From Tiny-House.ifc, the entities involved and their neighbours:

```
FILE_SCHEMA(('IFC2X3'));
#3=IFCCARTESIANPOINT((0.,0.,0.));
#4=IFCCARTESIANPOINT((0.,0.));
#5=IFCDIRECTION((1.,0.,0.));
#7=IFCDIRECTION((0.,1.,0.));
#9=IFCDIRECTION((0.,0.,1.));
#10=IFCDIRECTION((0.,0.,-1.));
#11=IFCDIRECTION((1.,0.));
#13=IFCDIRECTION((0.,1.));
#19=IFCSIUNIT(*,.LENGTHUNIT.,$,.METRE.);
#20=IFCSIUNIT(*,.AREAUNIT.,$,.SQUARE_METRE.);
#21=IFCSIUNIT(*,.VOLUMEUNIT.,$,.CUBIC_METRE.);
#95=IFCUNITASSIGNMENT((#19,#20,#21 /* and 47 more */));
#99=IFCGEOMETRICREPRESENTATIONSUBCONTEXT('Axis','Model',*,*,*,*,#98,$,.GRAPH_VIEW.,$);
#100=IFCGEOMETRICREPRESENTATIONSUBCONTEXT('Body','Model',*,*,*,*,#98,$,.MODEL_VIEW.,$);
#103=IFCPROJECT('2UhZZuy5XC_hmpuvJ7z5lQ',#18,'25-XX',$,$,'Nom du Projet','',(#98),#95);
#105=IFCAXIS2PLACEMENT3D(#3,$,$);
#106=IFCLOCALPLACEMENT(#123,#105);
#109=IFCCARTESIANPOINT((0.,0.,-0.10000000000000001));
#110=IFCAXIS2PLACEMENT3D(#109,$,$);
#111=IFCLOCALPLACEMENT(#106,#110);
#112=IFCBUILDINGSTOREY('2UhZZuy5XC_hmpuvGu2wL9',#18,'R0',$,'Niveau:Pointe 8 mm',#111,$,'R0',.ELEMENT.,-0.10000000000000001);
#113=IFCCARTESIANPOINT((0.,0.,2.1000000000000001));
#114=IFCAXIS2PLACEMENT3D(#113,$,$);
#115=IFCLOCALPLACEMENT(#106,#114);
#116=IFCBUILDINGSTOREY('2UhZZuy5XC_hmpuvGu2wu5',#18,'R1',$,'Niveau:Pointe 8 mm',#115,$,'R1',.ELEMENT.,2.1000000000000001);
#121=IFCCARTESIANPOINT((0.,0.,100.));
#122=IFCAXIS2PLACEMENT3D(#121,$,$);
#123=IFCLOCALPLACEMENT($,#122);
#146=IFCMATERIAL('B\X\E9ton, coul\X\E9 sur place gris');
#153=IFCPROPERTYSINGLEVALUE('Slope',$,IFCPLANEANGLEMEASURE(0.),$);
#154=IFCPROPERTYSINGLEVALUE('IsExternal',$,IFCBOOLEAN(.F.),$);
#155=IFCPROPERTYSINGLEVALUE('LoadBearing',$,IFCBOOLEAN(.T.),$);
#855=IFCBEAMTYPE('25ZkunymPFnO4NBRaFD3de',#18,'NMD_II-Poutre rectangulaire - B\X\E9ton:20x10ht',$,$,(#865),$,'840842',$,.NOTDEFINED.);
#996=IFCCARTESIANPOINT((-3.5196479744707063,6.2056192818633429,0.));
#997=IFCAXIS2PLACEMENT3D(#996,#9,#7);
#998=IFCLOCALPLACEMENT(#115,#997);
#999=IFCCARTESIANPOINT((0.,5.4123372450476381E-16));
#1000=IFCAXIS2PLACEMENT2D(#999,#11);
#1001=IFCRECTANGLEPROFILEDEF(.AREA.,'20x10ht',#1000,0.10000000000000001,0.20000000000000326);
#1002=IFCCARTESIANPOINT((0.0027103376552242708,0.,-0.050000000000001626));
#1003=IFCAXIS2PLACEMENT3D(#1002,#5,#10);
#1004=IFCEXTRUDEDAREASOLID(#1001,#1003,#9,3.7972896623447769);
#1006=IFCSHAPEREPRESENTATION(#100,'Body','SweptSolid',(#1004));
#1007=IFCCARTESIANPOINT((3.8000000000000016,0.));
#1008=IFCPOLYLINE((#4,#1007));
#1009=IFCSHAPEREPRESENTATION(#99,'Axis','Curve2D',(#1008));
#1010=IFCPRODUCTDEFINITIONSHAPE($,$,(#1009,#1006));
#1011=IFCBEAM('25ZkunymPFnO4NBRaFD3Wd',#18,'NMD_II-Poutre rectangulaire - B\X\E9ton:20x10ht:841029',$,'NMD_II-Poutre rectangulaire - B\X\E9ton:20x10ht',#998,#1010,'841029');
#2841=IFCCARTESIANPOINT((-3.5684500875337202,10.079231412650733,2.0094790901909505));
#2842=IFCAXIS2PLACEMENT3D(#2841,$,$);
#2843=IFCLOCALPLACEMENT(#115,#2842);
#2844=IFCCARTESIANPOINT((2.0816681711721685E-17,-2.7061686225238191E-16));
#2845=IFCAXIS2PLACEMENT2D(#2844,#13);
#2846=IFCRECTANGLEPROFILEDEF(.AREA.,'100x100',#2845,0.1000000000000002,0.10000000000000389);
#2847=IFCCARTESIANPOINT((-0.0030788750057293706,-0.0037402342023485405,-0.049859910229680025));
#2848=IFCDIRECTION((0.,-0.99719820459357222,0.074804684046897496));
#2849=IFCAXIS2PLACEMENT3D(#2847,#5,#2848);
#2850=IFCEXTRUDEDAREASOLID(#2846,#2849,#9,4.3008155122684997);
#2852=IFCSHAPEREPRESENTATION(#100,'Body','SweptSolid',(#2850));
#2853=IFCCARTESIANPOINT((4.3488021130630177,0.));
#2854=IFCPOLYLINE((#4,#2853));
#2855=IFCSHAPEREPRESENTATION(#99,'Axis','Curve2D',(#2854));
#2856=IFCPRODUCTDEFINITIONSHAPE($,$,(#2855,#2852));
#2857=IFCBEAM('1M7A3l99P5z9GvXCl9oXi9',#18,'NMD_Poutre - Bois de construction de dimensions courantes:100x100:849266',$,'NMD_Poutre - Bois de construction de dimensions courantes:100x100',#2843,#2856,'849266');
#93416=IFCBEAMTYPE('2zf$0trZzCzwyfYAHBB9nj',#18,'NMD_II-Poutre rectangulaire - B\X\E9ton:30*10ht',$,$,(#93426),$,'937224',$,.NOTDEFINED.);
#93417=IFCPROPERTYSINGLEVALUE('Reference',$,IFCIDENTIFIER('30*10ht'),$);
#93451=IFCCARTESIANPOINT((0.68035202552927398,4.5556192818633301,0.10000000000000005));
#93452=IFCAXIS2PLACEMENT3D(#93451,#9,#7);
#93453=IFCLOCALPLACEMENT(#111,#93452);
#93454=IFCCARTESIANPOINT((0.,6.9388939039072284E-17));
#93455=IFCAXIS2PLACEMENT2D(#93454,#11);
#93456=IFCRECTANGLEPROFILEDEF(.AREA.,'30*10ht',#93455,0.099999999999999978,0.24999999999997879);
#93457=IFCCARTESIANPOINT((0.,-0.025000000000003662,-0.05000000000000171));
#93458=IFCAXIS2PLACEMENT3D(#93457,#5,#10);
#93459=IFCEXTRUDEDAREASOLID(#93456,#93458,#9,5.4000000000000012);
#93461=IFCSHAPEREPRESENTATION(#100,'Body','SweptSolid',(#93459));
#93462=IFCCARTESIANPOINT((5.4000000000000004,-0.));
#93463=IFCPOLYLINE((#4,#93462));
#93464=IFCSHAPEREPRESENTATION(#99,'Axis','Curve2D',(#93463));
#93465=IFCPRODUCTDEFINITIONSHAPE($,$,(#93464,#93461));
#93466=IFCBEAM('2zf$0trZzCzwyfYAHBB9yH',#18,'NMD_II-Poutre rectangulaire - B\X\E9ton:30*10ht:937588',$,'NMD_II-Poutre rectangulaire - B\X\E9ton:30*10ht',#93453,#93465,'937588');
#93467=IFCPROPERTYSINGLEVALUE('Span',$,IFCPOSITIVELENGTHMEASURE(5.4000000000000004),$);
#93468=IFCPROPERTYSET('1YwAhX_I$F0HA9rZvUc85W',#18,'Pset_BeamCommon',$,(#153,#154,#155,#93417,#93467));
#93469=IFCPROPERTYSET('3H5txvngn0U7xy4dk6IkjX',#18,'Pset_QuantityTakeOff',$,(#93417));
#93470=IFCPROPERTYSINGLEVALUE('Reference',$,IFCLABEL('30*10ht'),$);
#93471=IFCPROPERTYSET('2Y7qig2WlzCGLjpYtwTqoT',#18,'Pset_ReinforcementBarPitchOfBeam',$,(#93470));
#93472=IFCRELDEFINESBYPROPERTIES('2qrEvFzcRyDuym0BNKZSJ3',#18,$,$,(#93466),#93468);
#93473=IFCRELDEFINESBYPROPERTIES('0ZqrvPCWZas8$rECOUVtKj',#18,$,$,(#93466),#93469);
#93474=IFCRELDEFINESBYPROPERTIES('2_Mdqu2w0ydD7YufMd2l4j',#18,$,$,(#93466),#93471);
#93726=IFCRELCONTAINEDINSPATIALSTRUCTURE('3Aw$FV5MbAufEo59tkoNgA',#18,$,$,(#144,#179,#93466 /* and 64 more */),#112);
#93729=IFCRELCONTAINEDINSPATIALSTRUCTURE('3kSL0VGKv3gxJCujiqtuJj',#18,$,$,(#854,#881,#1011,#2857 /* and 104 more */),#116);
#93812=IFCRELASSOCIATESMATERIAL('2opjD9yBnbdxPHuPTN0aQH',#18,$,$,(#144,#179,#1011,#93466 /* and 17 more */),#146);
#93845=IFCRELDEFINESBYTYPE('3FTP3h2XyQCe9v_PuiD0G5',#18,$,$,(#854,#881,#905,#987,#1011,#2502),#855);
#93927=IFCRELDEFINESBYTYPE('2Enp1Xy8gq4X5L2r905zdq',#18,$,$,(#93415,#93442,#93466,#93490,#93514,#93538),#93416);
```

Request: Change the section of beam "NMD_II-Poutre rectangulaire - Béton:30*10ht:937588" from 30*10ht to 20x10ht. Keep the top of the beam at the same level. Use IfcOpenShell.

```python
import ifcopenshell
import ifcopenshell.api.pset
import ifcopenshell.api.type
import ifcopenshell.util.element
import ifcopenshell.util.representation

model = ifcopenshell.open("Tiny-House.ifc")

member = model.by_id(93466)
source = next(p for p in model.by_type("IfcRectangleProfileDef") if p.ProfileName == "20x10ht")

body = ifcopenshell.util.representation.get_representation(member, "Model", "Body")
solid = body.Items[0]
old_profile = solid.SweptArea

# Copy the section's sizes but keep this member's own profile position.
profile = ifcopenshell.util.element.copy(model, source)
# Profiles are centred, so shift by half the change in depth to hold the top.
shift = (old_profile.XDim - profile.XDim) / 2
x, y = old_profile.Position.Location.Coordinates
up = (-1.0, 0.0)  # upwards, in the solid's own plane
location = model.createIfcCartesianPoint((x + up[0] * shift, y + up[1] * shift))
profile.Position = model.createIfcAxis2Placement2D(location, old_profile.Position.RefDirection)
solid.SweptArea = profile
if not model.get_total_inverses(old_profile):
    ifcopenshell.util.element.remove_deep2(model, old_profile)

new_type = model.by_guid("25ZkunymPFnO4NBRaFD3de")
ifcopenshell.api.type.assign_type(
    model, related_objects=[member], relating_type=new_type, should_map_representations=False
)
member.Name = member.Name.replace("30*10ht", "20x10ht")
member.ObjectType = "NMD_II-Poutre rectangulaire - Béton:20x10ht"
pset = model.by_id(ifcopenshell.util.element.get_pset(member, "Pset_BeamCommon", should_inherit=False)["id"])
ifcopenshell.api.pset.edit_pset(model, pset=pset, properties={"Reference": "20x10ht"})
pset = model.by_id(ifcopenshell.util.element.get_pset(member, "Pset_QuantityTakeOff", should_inherit=False)["id"])
ifcopenshell.api.pset.edit_pset(model, pset=pset, properties={"Reference": "20x10ht"})
pset = model.by_id(ifcopenshell.util.element.get_pset(member, "Pset_ReinforcementBarPitchOfBeam", should_inherit=False)["id"])
ifcopenshell.api.pset.edit_pset(model, pset=pset, properties={"Reference": "20x10ht"})

print(solid.SweptArea)

model.write("Tiny-House_rev.ifc")
```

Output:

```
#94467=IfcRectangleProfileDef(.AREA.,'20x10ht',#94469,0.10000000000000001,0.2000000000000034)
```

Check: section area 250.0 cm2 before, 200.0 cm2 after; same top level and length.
